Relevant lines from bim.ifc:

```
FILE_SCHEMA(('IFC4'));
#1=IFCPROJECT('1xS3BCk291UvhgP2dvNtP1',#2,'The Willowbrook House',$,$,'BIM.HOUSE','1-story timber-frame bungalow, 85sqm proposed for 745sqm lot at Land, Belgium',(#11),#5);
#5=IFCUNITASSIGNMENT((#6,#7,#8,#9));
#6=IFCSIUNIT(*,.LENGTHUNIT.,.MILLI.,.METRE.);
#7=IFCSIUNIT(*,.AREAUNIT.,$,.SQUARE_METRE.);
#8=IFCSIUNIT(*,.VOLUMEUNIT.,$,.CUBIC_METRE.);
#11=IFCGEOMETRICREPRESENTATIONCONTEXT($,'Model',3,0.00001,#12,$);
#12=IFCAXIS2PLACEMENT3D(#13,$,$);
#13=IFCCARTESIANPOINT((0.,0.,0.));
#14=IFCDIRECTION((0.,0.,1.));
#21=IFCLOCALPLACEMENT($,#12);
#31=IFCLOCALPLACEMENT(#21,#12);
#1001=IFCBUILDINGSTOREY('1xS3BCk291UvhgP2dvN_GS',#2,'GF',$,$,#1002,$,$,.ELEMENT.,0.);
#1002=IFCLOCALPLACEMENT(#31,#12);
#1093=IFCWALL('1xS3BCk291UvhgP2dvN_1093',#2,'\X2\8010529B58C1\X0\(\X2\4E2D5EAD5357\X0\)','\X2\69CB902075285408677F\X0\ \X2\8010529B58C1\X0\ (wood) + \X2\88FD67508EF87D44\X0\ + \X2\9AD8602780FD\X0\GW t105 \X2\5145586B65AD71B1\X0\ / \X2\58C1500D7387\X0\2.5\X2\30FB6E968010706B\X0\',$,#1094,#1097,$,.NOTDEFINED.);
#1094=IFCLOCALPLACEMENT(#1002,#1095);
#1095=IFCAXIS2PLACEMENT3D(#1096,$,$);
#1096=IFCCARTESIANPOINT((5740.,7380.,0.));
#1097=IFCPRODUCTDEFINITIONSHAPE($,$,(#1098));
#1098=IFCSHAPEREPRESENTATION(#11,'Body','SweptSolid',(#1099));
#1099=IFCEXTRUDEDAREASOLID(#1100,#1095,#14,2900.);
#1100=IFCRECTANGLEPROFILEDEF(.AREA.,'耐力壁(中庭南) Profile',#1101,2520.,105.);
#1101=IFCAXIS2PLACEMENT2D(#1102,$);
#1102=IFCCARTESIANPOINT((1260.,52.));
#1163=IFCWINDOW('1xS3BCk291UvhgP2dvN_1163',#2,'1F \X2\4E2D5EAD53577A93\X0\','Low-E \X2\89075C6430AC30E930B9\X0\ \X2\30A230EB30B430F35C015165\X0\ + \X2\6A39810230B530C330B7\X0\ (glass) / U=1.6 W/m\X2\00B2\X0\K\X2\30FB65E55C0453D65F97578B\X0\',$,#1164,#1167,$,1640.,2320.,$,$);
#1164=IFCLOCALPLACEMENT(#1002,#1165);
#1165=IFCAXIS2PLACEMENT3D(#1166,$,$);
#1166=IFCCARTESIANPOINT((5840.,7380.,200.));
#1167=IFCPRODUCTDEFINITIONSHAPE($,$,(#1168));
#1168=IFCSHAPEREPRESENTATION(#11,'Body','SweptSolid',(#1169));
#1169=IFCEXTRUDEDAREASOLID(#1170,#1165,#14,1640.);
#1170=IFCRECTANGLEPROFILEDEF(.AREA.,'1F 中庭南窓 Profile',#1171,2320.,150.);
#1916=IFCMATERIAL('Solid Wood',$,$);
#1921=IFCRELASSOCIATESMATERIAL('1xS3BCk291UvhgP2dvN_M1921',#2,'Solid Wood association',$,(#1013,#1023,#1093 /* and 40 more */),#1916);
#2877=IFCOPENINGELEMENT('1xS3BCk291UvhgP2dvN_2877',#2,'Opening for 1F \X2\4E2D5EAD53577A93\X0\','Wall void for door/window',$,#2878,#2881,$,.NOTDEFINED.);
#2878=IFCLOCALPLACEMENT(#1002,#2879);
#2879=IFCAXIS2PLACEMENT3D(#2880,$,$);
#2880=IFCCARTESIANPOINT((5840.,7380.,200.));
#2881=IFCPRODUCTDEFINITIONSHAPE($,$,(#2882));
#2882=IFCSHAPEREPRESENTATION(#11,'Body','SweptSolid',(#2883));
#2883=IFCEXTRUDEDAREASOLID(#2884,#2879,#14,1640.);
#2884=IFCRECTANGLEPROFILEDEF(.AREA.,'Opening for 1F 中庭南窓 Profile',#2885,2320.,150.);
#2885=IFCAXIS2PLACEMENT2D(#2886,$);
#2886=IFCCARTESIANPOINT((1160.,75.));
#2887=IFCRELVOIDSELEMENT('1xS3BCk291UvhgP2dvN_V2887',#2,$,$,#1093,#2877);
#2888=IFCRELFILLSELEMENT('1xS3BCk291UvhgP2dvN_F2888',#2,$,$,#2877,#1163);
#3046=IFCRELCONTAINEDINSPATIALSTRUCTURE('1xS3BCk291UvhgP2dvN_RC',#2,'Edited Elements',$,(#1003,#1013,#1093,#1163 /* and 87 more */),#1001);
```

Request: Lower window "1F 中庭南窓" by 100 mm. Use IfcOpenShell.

```python
import numpy as np
import ifcopenshell
import ifcopenshell.api.geometry
import ifcopenshell.util.placement
import ifcopenshell.util.unit

model = ifcopenshell.open("bim.ifc")
unit_scale = ifcopenshell.util.unit.calculate_unit_scale(model)

window = model.by_guid("1xS3BCk291UvhgP2dvN_1163")
opening = window.FillsVoids[0].RelatingOpeningElement
dz = -0.1 / unit_scale

shift = np.array([0.0, 0.0, dz])
# The window is not placed relative to its opening, so move both.
for product in (opening, window):
    matrix = ifcopenshell.util.placement.get_local_placement(product.ObjectPlacement)
    matrix[:3, 3] += shift
    ifcopenshell.api.geometry.edit_object_placement(model, product=product, matrix=matrix, is_si=False)

print(f"moved by {dz * unit_scale:+.3f} m")

model.write("bim-out.ifc")
```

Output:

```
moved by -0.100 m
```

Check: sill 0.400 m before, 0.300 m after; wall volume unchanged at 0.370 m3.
